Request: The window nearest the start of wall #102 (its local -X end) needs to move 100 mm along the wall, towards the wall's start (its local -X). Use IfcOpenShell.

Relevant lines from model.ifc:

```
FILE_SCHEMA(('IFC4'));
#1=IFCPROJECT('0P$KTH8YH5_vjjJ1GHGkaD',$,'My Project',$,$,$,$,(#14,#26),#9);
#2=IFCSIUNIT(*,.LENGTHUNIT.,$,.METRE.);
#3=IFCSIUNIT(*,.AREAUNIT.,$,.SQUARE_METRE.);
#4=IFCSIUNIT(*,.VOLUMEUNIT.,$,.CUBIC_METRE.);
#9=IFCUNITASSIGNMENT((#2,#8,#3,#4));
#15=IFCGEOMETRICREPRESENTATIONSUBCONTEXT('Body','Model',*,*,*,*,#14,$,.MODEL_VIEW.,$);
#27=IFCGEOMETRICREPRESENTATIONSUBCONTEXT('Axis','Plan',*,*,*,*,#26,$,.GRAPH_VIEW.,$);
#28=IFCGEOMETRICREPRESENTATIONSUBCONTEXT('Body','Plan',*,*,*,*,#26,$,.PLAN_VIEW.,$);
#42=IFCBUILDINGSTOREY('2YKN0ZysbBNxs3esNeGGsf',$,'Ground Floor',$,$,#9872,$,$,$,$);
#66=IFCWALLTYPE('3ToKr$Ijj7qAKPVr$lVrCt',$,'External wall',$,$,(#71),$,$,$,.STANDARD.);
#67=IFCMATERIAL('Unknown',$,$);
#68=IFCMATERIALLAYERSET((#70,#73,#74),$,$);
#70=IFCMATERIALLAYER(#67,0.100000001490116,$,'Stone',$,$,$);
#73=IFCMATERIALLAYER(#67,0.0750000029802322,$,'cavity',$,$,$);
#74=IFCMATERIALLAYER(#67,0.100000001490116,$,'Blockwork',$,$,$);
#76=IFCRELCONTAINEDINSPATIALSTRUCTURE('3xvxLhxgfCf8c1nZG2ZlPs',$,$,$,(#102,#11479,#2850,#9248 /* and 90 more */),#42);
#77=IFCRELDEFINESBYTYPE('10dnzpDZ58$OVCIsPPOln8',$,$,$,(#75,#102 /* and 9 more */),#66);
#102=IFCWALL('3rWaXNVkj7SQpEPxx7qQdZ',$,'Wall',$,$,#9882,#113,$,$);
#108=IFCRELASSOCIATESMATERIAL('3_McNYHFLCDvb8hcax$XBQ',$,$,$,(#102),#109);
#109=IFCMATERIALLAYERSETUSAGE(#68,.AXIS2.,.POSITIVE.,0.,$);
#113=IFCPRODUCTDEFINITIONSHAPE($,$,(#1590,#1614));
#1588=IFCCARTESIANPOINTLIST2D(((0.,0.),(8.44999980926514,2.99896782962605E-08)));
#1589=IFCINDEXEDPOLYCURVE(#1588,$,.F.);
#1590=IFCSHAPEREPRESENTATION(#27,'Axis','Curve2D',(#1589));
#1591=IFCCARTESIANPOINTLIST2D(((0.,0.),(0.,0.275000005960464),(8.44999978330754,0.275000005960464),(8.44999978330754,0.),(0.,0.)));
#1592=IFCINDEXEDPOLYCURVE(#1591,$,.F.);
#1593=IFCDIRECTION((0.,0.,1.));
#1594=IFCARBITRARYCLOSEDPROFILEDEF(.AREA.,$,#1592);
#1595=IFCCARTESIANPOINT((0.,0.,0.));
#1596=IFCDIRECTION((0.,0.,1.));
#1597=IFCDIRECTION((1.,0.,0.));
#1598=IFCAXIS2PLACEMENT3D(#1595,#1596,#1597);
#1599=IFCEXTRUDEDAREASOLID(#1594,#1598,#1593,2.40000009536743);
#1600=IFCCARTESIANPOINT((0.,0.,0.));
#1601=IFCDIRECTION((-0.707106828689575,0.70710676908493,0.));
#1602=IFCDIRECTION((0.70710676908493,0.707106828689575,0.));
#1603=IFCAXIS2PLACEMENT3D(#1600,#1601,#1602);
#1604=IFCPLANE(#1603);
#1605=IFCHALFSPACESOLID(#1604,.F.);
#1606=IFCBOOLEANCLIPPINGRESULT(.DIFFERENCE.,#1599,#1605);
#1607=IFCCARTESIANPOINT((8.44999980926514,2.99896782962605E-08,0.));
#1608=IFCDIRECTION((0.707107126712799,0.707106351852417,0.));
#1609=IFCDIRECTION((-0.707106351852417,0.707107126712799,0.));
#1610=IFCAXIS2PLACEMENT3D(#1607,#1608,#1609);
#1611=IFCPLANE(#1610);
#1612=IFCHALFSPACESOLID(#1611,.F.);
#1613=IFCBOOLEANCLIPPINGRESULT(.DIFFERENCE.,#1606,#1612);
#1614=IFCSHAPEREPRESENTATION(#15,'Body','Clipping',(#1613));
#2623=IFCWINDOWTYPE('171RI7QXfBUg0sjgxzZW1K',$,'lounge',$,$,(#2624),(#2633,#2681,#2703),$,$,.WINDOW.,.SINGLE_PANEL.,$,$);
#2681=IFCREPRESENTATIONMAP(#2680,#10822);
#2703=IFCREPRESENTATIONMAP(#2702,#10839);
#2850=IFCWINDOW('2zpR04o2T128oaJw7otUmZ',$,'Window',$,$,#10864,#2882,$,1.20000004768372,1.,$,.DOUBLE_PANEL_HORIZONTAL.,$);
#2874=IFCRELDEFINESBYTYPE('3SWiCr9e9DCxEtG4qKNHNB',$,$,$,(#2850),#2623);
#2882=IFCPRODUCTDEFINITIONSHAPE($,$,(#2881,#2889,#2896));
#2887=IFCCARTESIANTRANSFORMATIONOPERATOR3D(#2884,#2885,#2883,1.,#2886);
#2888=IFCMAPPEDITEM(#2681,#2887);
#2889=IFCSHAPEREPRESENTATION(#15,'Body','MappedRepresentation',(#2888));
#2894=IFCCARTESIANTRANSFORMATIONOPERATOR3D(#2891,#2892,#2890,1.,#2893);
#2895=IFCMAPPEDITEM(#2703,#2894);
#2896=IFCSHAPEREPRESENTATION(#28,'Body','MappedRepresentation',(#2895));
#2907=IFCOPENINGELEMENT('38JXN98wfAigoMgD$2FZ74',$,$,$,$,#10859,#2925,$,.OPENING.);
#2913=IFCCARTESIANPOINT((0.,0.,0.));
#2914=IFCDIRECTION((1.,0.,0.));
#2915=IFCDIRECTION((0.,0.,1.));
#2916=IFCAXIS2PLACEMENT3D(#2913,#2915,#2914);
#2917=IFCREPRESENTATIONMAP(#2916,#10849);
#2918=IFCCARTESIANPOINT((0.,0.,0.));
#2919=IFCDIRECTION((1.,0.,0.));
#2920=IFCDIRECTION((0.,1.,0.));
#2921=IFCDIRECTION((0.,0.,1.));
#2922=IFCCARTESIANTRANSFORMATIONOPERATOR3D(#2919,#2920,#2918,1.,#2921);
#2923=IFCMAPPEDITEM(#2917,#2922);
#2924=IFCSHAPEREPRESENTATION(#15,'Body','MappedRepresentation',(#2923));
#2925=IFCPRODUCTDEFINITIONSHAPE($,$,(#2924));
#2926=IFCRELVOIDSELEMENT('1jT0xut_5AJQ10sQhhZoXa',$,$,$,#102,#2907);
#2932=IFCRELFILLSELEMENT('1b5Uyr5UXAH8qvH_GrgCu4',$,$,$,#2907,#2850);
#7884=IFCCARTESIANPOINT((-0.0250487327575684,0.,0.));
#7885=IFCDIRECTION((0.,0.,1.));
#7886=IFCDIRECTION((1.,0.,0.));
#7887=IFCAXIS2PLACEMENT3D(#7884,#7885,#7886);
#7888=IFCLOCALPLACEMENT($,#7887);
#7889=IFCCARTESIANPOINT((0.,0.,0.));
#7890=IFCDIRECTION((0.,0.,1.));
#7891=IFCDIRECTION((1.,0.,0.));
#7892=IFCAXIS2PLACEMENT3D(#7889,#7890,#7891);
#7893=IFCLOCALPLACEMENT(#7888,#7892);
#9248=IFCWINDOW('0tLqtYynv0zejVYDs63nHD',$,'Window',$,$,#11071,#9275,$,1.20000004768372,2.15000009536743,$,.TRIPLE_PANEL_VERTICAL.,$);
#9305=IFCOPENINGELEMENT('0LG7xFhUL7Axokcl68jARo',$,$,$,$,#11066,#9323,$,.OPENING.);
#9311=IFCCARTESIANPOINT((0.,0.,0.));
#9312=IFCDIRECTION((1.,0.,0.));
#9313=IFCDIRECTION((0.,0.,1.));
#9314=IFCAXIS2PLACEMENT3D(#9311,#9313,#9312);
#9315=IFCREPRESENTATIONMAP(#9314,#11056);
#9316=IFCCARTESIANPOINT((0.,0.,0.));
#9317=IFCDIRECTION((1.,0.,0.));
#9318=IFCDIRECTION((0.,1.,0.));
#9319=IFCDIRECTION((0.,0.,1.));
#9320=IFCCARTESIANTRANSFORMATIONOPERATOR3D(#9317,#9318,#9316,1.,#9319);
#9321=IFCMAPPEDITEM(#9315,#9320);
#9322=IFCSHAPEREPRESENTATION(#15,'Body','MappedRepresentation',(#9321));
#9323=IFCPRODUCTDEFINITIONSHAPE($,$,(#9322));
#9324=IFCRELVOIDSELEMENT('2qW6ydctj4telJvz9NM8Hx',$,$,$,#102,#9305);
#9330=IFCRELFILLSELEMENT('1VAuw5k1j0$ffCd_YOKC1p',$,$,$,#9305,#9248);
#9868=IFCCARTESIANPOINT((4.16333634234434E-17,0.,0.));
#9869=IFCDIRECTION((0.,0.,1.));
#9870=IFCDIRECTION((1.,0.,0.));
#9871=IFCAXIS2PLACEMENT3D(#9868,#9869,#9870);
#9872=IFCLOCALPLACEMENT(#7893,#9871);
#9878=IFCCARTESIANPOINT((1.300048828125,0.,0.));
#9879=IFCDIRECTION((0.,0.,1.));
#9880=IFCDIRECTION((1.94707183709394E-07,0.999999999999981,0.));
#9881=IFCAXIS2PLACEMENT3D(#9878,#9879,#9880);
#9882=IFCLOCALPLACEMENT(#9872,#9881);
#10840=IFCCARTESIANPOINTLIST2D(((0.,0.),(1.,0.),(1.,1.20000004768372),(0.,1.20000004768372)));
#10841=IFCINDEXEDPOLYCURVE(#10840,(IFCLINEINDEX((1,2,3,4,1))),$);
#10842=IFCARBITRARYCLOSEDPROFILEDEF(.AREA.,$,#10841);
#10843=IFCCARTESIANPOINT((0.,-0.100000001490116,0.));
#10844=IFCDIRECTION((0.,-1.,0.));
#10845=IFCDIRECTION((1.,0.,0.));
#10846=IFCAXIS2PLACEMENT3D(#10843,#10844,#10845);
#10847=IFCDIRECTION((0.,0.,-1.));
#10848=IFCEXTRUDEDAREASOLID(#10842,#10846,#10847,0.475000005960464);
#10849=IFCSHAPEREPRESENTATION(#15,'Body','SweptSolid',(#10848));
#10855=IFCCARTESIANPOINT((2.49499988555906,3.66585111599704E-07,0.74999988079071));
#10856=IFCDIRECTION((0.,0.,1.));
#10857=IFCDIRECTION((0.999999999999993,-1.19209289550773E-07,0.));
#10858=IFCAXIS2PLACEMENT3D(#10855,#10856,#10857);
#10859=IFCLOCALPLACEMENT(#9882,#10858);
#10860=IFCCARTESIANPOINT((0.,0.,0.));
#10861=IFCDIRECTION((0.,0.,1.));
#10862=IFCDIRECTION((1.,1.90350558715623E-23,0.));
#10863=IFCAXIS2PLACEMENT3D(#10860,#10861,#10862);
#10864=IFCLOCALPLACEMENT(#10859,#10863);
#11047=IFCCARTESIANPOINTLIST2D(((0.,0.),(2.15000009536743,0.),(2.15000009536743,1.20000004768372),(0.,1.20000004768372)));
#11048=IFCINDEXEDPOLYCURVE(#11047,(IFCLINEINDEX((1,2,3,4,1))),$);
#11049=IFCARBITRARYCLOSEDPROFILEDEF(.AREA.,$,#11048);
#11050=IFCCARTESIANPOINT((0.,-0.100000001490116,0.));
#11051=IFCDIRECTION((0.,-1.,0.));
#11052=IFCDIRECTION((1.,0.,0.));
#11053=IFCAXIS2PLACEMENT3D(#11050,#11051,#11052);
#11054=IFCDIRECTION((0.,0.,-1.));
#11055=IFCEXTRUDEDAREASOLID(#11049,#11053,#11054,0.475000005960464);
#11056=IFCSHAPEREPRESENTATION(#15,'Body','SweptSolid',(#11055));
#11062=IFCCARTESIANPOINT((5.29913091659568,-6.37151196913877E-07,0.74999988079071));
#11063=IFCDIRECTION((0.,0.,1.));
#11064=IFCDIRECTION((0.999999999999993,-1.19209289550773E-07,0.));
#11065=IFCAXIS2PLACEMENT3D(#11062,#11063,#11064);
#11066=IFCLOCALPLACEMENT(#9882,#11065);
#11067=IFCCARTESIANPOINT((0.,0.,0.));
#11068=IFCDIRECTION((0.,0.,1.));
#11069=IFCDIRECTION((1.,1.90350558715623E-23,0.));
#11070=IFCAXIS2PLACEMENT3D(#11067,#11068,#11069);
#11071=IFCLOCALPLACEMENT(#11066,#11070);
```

```python
import ifcopenshell
import ifcopenshell.api.geometry
import ifcopenshell.util.placement
import ifcopenshell.util.unit

model = ifcopenshell.open("model.ifc")
unit_scale = ifcopenshell.util.unit.calculate_unit_scale(model)

window = model.by_guid("2zpR04o2T128oaJw7otUmZ")
opening = window.FillsVoids[0].RelatingOpeningElement
wall = opening.VoidsElements[0].RelatingBuildingElement

wall_matrix = ifcopenshell.util.placement.get_local_placement(wall.ObjectPlacement)
shift = wall_matrix[:3, 0] * -0.1 / unit_scale
before = ifcopenshell.util.placement.get_local_placement(window.ObjectPlacement)[:3, 3].copy()

# The window is placed relative to its opening, so it follows when the opening moves.
matrix = ifcopenshell.util.placement.get_local_placement(opening.ObjectPlacement)
matrix[:3, 3] += shift
ifcopenshell.api.geometry.edit_object_placement(
    model, product=opening, matrix=matrix, is_si=False, should_transform_children=True
)

after = ifcopenshell.util.placement.get_local_placement(window.ObjectPlacement)[:3, 3]
print("window moved by", (after - before).round(3) + 0.0)

model.write("model_updated.ifc")
```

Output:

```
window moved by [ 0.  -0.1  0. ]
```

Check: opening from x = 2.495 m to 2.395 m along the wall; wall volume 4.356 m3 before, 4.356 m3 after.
